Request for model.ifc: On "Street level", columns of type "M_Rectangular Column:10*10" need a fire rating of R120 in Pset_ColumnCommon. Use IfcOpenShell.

First a look at what the model holds.

```python
import ifcopenshell
import ifcopenshell.util.element

model = ifcopenshell.open("model.ifc")
print(model.schema)
storey = next(s for s in model.by_type("IfcBuildingStorey") if s.Name == "Street level")
columns = [e for e in ifcopenshell.util.element.get_decomposition(storey) if e.is_a("IfcColumn")]
seen = {}
for e in columns:
    element_type = ifcopenshell.util.element.get_type(e)
    key = (element_type.Name if element_type != e and element_type else None, ifcopenshell.util.element.get_pset(e, "Pset_ColumnCommon", "FireRating"))
    seen[key] = seen.get(key, 0) + 1
for (name, value), count in sorted(seen.items(), key=str):
    print(count, "x", name, "|", value)
```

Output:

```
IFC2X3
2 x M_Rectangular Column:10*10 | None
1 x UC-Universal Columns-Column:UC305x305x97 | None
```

```python
import ifcopenshell
import ifcopenshell.api.pset
import ifcopenshell.util.element

model = ifcopenshell.open("model.ifc")

storey = next(s for s in model.by_type("IfcBuildingStorey") if s.Name == "Street level")
columns = [e for e in ifcopenshell.util.element.get_decomposition(storey) if e.is_a("IfcColumn")]

count = 0
for e in columns:
    element_type = ifcopenshell.util.element.get_type(e)
    if element_type in (None, e) or element_type.Name != "M_Rectangular Column:10*10":
        continue
    # add_pset returns the element's existing set when there is one.
    pset = ifcopenshell.api.pset.add_pset(model, product=e, name="Pset_ColumnCommon")
    ifcopenshell.api.pset.edit_pset(model, pset=pset, properties={"FireRating": "R120"})
    count += 1

print(count, "columns updated")

model.write("model-out.ifc")
```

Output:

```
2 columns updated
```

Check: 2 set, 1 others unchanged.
